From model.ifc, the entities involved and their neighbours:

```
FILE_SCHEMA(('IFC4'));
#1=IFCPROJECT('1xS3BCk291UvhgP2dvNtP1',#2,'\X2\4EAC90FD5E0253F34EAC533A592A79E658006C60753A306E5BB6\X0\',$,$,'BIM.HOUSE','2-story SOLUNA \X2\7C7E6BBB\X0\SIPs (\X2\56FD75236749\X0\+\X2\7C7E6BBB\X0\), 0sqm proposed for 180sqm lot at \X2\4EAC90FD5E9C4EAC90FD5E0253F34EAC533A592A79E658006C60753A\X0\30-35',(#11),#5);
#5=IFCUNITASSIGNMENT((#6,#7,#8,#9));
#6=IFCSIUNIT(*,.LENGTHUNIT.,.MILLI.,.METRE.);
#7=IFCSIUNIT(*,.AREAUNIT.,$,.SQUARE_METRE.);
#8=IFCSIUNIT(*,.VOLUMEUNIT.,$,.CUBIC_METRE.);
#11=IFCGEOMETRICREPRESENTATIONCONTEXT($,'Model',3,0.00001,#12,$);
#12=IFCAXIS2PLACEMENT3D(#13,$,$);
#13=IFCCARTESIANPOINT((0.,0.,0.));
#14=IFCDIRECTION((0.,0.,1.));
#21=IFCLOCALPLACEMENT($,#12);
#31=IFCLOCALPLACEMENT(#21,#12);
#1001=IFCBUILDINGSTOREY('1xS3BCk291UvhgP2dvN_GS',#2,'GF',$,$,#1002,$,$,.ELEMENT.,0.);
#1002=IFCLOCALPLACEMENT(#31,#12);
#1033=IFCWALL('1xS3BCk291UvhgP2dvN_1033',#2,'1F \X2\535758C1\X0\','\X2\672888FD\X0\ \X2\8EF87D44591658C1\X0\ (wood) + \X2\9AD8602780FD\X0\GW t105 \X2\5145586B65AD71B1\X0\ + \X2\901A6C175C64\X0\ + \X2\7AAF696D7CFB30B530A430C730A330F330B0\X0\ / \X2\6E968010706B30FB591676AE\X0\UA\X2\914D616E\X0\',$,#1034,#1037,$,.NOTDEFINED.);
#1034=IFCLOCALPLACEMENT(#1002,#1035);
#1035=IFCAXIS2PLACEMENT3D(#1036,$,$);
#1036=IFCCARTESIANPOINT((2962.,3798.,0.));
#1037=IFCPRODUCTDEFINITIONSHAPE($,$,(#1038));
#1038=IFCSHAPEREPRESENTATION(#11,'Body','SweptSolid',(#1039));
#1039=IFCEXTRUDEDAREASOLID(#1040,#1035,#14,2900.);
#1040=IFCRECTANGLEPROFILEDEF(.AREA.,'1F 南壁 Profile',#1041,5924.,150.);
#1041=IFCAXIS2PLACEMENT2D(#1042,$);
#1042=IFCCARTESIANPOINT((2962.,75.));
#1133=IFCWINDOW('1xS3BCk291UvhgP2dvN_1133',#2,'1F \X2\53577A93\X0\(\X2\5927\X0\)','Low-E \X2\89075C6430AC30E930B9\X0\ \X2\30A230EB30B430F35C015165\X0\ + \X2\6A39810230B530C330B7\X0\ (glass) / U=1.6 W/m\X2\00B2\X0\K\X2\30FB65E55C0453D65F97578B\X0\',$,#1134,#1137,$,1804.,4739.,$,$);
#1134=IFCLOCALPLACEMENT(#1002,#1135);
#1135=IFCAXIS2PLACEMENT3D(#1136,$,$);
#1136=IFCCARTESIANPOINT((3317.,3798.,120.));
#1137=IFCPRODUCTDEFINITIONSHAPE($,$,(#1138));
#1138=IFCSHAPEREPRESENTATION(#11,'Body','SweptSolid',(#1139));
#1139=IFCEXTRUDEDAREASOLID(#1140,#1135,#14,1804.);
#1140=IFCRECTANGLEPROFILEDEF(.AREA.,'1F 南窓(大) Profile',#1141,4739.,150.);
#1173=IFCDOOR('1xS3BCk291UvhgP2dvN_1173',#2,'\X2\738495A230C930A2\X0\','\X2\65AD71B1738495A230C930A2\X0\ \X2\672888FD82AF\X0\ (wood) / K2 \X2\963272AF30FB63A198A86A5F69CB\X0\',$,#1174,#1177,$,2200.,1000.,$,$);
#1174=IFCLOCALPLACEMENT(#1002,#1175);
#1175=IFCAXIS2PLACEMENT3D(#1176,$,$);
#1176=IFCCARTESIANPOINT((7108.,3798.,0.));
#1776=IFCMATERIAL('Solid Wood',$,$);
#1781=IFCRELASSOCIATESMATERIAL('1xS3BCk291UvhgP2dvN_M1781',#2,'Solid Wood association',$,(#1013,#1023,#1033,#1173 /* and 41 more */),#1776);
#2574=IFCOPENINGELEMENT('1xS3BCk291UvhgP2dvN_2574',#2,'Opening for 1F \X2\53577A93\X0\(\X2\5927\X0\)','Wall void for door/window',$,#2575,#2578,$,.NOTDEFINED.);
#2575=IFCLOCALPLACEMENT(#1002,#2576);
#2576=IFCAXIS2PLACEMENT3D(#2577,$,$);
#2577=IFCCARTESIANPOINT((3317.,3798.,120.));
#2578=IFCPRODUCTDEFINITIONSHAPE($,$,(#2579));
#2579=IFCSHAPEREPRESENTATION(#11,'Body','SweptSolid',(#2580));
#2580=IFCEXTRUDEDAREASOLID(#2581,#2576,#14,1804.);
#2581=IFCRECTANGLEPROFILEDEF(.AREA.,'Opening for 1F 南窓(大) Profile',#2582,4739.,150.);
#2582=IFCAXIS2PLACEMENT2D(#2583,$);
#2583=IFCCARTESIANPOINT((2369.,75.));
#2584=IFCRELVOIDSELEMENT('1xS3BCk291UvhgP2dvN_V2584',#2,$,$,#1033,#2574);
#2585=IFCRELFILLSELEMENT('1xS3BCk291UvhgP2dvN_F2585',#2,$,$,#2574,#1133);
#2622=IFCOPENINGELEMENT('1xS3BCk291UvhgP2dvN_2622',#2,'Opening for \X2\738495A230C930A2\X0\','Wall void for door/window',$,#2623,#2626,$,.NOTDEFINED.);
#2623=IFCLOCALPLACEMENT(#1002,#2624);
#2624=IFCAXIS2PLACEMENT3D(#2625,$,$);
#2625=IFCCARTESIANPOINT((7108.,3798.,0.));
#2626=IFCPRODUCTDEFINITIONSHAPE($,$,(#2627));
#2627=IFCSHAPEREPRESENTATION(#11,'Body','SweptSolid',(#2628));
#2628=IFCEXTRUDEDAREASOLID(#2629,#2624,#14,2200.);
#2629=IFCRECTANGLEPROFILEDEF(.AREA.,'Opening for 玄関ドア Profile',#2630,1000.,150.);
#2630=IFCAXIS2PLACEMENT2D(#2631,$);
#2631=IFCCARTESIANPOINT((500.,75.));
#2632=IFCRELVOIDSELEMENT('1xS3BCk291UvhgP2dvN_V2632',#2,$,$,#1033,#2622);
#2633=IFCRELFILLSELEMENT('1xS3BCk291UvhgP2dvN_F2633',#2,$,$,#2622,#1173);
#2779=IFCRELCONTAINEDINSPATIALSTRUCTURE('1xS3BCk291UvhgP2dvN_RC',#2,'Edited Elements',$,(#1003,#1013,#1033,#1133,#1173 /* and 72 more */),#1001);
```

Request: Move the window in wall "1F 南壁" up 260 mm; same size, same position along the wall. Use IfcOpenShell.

```python
import numpy as np
import ifcopenshell
import ifcopenshell.api.geometry
import ifcopenshell.util.placement
import ifcopenshell.util.unit

model = ifcopenshell.open("model.ifc")
unit_scale = ifcopenshell.util.unit.calculate_unit_scale(model)

window = model.by_guid("1xS3BCk291UvhgP2dvN_1133")
opening = window.FillsVoids[0].RelatingOpeningElement
dz = 260.0

shift = np.array([0.0, 0.0, dz])
# The window is not placed relative to its opening, so move both.
for product in (opening, window):
    matrix = ifcopenshell.util.placement.get_local_placement(product.ObjectPlacement)
    matrix[:3, 3] += shift
    ifcopenshell.api.geometry.edit_object_placement(model, product=product, matrix=matrix, is_si=False)

print(f"moved by {dz * unit_scale:+.3f} m")

model.write("model-out.ifc")
```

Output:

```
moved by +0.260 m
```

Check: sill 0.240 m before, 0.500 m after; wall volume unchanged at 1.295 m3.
